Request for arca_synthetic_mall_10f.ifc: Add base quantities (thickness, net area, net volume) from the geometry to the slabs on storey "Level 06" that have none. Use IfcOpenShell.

First a look at what the model holds.

```python
import ifcopenshell
import ifcopenshell.util.element
import ifcopenshell.util.unit

model = ifcopenshell.open("arca_synthetic_mall_10f.ifc")
print(model.schema)
for unit_type in ("LENGTHUNIT", "AREAUNIT", "VOLUMEUNIT"):
    print(unit_type, ifcopenshell.util.unit.calculate_unit_scale(model, unit_type))
storey = next(s for s in model.by_type("IfcBuildingStorey") if s.Name == "Level 06")
slabs = [e for e in ifcopenshell.util.element.get_decomposition(storey) if e.is_a("IfcSlab")]
for e in sorted(slabs, key=lambda e: e.id()):
    print(e.id(), e.is_a(), e.Name, list(ifcopenshell.util.element.get_psets(e, qtos_only=True)), sep=" | ")
```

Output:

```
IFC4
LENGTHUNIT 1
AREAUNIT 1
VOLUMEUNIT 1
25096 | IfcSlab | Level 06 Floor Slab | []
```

```python
import ifcopenshell
import ifcopenshell.api.pset
import ifcopenshell.geom
import ifcopenshell.util.element
import ifcopenshell.util.shape
import ifcopenshell.util.unit

model = ifcopenshell.open("arca_synthetic_mall_10f.ifc")
unit_scale = ifcopenshell.util.unit.calculate_unit_scale(model)
area_scale = ifcopenshell.util.unit.calculate_unit_scale(model, "AREAUNIT")
volume_scale = ifcopenshell.util.unit.calculate_unit_scale(model, "VOLUMEUNIT")
settings = ifcopenshell.geom.settings()

storey = next(s for s in model.by_type("IfcBuildingStorey") if s.Name == "Level 06")
slabs = [e for e in ifcopenshell.util.element.get_decomposition(storey) if e.is_a("IfcSlab")]

for e in sorted(slabs, key=lambda e: e.id()):
    if ifcopenshell.util.element.get_psets(e, qtos_only=True, should_inherit=False):
        continue
    # Geometry comes back in metres, in the element's own axes.
    shape = ifcopenshell.geom.create_shape(settings, e)
    values = {
        "Width": ifcopenshell.util.shape.get_z(shape.geometry) / unit_scale,
        "NetArea": ifcopenshell.util.shape.get_footprint_area(shape.geometry) / area_scale,
        "NetVolume": ifcopenshell.util.shape.get_volume(shape.geometry) / volume_scale,
    }
    qto = ifcopenshell.api.pset.add_qto(model, product=e, name="Qto_SlabBaseQuantities")
    ifcopenshell.api.pset.edit_qto(model, qto=qto, properties=values)
    print(e.id(), {k: round(v, 3) for k, v in values.items()})

model.write("arca_synthetic_mall_10f_rev.ifc")
```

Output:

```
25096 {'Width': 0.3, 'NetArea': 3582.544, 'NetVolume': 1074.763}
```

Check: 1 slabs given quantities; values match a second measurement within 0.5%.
